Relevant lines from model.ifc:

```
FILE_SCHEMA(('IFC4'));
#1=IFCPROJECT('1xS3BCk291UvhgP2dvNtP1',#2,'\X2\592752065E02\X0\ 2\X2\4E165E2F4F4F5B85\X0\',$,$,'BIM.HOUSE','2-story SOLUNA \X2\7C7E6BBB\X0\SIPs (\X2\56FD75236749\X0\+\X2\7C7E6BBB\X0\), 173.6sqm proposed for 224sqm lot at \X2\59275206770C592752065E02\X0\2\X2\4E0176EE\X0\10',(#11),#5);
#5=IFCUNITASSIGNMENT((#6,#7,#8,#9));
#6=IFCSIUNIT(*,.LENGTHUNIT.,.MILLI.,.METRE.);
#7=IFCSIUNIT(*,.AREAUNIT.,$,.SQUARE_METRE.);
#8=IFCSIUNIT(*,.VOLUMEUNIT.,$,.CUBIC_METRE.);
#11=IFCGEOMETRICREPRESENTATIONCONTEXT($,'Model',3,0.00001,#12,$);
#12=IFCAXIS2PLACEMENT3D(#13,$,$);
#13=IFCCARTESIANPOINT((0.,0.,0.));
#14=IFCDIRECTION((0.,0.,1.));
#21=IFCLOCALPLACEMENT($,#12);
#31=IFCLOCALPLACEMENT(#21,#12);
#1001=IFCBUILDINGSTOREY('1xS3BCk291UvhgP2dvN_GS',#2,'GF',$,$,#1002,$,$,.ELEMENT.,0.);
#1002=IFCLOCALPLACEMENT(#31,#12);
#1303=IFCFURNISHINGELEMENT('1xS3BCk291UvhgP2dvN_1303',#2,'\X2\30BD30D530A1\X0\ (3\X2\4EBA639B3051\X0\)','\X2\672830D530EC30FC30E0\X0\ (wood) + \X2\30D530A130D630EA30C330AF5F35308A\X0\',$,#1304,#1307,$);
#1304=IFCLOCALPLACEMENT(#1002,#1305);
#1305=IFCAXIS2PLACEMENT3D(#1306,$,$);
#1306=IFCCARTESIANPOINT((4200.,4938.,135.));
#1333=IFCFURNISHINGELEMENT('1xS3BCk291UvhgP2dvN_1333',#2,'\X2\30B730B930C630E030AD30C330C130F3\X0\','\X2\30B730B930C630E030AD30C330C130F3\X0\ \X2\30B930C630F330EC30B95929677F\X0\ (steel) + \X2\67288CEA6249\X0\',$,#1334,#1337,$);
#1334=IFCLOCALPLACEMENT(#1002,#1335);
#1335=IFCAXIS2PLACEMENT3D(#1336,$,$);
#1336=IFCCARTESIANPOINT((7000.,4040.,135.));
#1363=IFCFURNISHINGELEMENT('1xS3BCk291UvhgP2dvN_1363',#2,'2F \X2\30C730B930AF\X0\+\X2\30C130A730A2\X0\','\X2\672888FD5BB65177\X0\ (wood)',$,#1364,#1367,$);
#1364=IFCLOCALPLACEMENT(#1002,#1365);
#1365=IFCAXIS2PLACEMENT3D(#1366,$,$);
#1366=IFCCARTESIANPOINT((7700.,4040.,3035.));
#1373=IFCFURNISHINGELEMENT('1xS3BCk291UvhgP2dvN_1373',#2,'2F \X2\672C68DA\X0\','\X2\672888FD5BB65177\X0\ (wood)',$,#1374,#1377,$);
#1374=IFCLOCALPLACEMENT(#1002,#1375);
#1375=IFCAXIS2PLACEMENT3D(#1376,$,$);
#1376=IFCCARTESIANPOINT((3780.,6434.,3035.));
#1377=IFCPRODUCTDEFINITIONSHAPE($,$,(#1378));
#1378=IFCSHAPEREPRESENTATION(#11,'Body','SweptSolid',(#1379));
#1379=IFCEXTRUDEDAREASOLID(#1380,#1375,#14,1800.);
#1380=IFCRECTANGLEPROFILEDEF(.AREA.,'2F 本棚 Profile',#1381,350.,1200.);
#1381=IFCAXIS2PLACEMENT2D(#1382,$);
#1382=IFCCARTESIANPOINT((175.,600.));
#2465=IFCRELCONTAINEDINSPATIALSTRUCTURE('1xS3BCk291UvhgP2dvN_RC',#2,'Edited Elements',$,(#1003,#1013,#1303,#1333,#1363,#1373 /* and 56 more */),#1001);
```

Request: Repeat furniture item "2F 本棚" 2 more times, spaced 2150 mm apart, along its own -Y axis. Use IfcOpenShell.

```python
import ifcopenshell
import ifcopenshell.api.geometry
import ifcopenshell.api.root
import ifcopenshell.util.element
import ifcopenshell.util.placement

model = ifcopenshell.open("model.ifc")


def reuse_history(source, copy):
    """copy_class also copies each property set's owner history, people and application; keep the originals."""
    for rel in copy.IsDefinedBy:
        if rel.is_a("IfcRelDefinesByProperties") and (history := rel.RelatingPropertyDefinition.OwnerHistory):
            rel.RelatingPropertyDefinition.OwnerHistory = source.OwnerHistory
            ifcopenshell.util.element.remove_deep2(model, history)


source = model.by_guid("1xS3BCk291UvhgP2dvN_1373")
base = ifcopenshell.util.placement.get_local_placement(source.ObjectPlacement)
step = -base[:3, 1] * 2150.0

for i in range(1, 3):
    copy = ifcopenshell.api.root.copy_class(model, product=source)
    copy.Representation = ifcopenshell.util.element.copy_deep(
        model, source.Representation, exclude=["IfcGeometricRepresentationContext", "IfcRepresentationMap"]
    )
    reuse_history(source, copy)
    matrix = base.copy()
    matrix[:3, 3] += i * step
    print("added at", matrix[:3, 3].round(3) + 0.0)
    ifcopenshell.api.geometry.edit_object_placement(model, product=copy, matrix=matrix, is_si=False)

model.write("model-out.ifc")
```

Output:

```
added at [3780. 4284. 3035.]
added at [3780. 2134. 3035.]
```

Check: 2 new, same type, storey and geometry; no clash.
